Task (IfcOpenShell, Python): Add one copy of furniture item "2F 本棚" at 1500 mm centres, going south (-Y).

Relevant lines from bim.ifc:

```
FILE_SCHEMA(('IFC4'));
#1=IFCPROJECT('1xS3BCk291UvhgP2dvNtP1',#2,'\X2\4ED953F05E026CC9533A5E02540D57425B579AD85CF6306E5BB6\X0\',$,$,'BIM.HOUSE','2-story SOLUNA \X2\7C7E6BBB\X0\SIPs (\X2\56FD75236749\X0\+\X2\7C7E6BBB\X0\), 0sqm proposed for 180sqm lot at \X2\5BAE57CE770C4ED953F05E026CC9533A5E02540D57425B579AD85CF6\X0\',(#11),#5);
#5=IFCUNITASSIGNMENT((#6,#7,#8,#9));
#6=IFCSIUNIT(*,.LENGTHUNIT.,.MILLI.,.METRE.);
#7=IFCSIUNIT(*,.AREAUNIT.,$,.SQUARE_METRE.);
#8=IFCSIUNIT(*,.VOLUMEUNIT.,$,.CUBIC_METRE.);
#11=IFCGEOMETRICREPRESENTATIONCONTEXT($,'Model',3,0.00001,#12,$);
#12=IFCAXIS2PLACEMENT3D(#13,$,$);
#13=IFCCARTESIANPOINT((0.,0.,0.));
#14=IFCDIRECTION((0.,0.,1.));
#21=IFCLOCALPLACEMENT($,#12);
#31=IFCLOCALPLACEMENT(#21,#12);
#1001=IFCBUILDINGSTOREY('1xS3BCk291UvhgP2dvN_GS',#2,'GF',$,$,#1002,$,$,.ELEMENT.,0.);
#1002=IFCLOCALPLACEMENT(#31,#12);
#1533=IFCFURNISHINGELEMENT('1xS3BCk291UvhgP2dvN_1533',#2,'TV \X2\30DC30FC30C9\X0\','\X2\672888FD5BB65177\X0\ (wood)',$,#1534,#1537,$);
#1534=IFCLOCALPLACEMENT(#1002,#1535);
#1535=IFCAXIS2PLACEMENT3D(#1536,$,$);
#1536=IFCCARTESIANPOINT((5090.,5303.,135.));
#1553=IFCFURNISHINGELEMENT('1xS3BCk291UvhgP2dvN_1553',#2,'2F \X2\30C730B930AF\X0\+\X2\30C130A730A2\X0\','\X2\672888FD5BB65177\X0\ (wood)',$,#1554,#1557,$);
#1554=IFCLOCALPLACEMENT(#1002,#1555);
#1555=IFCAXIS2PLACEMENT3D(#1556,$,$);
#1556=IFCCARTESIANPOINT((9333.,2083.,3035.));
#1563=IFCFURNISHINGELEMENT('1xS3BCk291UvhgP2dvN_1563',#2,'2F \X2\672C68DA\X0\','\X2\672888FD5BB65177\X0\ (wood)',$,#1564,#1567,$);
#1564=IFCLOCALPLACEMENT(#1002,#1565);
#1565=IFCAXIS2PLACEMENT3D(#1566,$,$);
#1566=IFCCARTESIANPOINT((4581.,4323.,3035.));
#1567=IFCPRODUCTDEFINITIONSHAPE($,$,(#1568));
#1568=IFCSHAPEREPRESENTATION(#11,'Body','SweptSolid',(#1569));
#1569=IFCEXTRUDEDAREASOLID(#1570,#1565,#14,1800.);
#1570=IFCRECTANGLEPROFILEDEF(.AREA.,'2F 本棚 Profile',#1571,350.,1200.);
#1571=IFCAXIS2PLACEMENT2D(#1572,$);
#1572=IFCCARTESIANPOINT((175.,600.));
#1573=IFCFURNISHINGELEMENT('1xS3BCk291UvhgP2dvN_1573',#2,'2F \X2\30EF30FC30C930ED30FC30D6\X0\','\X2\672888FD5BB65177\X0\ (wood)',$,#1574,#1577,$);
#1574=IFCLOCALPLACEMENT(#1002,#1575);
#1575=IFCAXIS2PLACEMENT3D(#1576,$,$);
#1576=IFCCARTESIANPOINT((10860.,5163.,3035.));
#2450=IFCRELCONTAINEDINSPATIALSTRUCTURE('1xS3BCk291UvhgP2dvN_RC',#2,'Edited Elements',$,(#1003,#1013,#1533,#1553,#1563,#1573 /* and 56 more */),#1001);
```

```python
import numpy as np
import ifcopenshell
import ifcopenshell.api.geometry
import ifcopenshell.api.root
import ifcopenshell.util.element
import ifcopenshell.util.placement

model = ifcopenshell.open("bim.ifc")


def reuse_history(source, copy):
    """copy_class also copies each property set's owner history, people and application; keep the originals."""
    for rel in copy.IsDefinedBy:
        if rel.is_a("IfcRelDefinesByProperties") and (history := rel.RelatingPropertyDefinition.OwnerHistory):
            rel.RelatingPropertyDefinition.OwnerHistory = source.OwnerHistory
            ifcopenshell.util.element.remove_deep2(model, history)


source = model.by_guid("1xS3BCk291UvhgP2dvN_1563")
base = ifcopenshell.util.placement.get_local_placement(source.ObjectPlacement)
step = np.array([0.0, -1.0, 0.0]) * 1500.0

for i in range(1, 2):
    copy = ifcopenshell.api.root.copy_class(model, product=source)
    copy.Representation = ifcopenshell.util.element.copy_deep(
        model, source.Representation, exclude=["IfcGeometricRepresentationContext", "IfcRepresentationMap"]
    )
    reuse_history(source, copy)
    matrix = base.copy()
    matrix[:3, 3] += i * step
    print("added at", matrix[:3, 3].round(3) + 0.0)
    ifcopenshell.api.geometry.edit_object_placement(model, product=copy, matrix=matrix, is_si=False)

model.write("bim_edited.ifc")
```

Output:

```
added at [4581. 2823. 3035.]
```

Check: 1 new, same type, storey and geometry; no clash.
